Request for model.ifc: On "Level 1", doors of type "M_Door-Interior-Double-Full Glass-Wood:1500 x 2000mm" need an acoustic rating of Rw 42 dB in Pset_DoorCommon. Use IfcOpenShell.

First a look at what the model holds.

```python
import ifcopenshell
import ifcopenshell.util.element

model = ifcopenshell.open("model.ifc")
print(model.schema)
storey = next(s for s in model.by_type("IfcBuildingStorey") if s.Name == "Level 1")
doors = [e for e in ifcopenshell.util.element.get_decomposition(storey) if e.is_a("IfcDoor")]
seen = {}
for e in doors:
    element_type = ifcopenshell.util.element.get_type(e)
    key = (element_type.Name if element_type != e and element_type else None, ifcopenshell.util.element.get_pset(e, "Pset_DoorCommon", "AcousticRating"))
    seen[key] = seen.get(key, 0) + 1
for (name, value), count in sorted(seen.items(), key=str):
    print(count, "x", name, "|", value)
```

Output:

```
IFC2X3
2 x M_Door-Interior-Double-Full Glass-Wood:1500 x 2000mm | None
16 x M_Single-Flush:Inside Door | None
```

```python
import ifcopenshell
import ifcopenshell.api.pset
import ifcopenshell.util.element

model = ifcopenshell.open("model.ifc")

storey = next(s for s in model.by_type("IfcBuildingStorey") if s.Name == "Level 1")
doors = [e for e in ifcopenshell.util.element.get_decomposition(storey) if e.is_a("IfcDoor")]

count = 0
for e in doors:
    element_type = ifcopenshell.util.element.get_type(e)
    if element_type in (None, e) or element_type.Name != "M_Door-Interior-Double-Full Glass-Wood:1500 x 2000mm":
        continue
    # add_pset returns the element's existing set when there is one.
    pset = ifcopenshell.api.pset.add_pset(model, product=e, name="Pset_DoorCommon")
    ifcopenshell.api.pset.edit_pset(model, pset=pset, properties={"AcousticRating": "Rw 42 dB"})
    count += 1

print(count, "doors updated")

model.write("model_v2.ifc")
```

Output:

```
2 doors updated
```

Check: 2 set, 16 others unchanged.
